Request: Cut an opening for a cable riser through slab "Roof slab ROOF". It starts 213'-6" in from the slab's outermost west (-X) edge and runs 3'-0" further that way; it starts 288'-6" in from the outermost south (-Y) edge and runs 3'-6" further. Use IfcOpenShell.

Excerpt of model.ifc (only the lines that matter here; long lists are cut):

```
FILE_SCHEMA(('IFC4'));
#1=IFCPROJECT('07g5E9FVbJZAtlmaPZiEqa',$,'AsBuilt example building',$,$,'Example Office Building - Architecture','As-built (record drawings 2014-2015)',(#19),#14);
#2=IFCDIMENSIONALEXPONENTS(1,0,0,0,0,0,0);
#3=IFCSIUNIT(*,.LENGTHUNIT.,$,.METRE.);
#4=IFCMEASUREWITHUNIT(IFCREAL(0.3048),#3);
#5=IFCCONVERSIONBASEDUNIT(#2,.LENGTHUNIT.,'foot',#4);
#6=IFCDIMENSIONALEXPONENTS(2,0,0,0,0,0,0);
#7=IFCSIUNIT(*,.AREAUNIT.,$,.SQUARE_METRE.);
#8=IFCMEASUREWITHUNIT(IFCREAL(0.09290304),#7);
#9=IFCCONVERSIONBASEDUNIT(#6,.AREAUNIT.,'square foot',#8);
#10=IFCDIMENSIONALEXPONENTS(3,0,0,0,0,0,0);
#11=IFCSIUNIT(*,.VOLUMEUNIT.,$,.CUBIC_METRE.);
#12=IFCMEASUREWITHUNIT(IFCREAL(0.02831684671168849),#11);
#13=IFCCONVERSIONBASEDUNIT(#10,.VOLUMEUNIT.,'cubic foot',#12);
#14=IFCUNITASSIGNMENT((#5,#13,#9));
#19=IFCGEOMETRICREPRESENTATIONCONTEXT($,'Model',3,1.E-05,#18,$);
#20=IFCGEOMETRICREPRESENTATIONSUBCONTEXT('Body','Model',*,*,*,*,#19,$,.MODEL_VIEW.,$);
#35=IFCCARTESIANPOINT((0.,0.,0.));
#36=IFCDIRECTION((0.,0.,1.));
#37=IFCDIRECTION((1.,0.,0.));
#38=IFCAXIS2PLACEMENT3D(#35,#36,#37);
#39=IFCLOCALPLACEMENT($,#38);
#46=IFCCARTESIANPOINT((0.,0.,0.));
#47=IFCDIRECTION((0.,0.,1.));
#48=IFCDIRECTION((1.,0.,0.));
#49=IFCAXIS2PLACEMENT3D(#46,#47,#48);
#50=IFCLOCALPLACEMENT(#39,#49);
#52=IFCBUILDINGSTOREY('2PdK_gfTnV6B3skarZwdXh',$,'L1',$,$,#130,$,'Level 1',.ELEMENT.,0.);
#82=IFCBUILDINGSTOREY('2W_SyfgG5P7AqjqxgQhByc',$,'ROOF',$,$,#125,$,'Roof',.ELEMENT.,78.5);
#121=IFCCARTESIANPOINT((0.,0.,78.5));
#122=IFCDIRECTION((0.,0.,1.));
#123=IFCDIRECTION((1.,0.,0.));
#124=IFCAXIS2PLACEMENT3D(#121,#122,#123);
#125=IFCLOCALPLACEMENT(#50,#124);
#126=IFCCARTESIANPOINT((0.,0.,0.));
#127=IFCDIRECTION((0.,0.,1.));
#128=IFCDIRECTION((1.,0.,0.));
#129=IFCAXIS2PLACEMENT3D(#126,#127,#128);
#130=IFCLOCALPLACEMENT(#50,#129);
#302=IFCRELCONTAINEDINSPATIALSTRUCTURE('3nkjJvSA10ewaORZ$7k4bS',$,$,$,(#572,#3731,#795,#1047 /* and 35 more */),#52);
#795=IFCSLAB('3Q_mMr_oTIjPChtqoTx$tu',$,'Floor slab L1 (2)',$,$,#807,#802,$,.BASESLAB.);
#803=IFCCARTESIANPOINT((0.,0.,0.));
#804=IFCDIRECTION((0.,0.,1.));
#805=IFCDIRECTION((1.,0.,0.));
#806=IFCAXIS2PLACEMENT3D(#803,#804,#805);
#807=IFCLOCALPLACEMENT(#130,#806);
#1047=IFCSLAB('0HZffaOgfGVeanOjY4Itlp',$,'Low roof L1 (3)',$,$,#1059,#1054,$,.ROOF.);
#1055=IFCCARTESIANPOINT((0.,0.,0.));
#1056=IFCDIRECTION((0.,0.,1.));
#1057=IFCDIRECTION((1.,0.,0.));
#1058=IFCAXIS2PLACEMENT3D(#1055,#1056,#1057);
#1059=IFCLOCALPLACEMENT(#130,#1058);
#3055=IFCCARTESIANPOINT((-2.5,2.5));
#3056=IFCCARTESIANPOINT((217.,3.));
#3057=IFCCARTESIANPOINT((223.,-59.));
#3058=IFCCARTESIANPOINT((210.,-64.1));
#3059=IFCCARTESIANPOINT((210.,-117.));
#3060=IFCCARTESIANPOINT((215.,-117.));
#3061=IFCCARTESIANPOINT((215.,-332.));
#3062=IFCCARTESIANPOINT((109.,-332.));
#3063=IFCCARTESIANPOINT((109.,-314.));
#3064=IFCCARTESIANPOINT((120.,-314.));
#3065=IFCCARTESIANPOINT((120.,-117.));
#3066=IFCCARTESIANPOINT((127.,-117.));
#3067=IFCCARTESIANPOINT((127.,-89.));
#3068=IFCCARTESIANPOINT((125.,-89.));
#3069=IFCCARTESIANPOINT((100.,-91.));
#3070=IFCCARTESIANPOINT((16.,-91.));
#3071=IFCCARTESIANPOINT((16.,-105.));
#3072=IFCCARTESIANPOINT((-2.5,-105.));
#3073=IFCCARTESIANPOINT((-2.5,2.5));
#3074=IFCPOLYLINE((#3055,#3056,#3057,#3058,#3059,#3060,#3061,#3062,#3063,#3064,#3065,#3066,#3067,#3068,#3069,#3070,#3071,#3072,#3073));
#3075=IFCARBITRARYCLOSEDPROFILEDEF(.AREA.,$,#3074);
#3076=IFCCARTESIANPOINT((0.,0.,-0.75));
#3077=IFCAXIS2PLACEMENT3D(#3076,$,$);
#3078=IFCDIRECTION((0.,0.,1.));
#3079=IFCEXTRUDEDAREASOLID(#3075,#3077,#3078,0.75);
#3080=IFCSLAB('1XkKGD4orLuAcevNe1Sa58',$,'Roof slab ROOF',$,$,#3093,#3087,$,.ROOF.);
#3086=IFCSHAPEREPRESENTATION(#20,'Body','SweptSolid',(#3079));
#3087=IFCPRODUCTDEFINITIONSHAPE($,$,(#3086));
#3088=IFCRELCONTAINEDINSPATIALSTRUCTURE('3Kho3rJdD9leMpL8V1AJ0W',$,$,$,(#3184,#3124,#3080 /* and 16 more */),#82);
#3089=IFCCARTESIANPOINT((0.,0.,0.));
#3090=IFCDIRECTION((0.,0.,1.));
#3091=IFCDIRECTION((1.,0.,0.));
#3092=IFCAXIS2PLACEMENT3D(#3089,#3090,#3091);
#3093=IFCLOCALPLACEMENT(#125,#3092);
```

```python
import numpy as np
import ifcopenshell
import ifcopenshell.api.feature
import ifcopenshell.api.geometry
import ifcopenshell.api.root
import ifcopenshell.geom
import ifcopenshell.util.placement
import ifcopenshell.util.representation
import ifcopenshell.util.shape
import ifcopenshell.util.unit

model = ifcopenshell.open("model.ifc")
unit_scale = ifcopenshell.util.unit.calculate_unit_scale(model)
settings = ifcopenshell.geom.settings()


def volume(element):
    """Net volume in cubic metres, openings subtracted."""
    shape = ifcopenshell.geom.create_shape(settings, element)
    return ifcopenshell.util.shape.get_volume(shape.geometry)


slab = model.by_guid("1XkKGD4orLuAcevNe1Sa58")
before = volume(slab)

# Extent in the slab's own axes, in metres. The edges named are its -X and -Y sides.
slab_shape = ifcopenshell.geom.create_shape(settings, slab)
vertices = ifcopenshell.util.shape.get_vertices(slab_shape.geometry)
x_min, y_min, bottom = vertices.min(axis=0)
top = vertices[:, 2].max()

opening = ifcopenshell.api.root.create_entity(model, ifc_class="IfcOpeningElement", name="Cable riser opening", predefined_type="OPENING")
context = ifcopenshell.util.representation.get_context(model, "Model", "Body", "MODEL_VIEW")
width, depth = 0.9144, 1.0668
outline = [(0.0, 0.0), (width, 0.0), (width, depth), (0.0, depth), (0.0, 0.0)]
# Overshoot both faces by 50 mm so the cut is clean.
shape = ifcopenshell.api.geometry.add_slab_representation(
    model, context=context, depth=top - bottom + 0.1, polyline=outline
)
ifcopenshell.api.geometry.assign_representation(model, product=opening, representation=shape)

matrix = ifcopenshell.util.placement.get_local_placement(slab.ObjectPlacement)
matrix[:, 3] = matrix @ np.append(np.array([x_min + 65.0748, y_min + 87.9348, bottom - 0.05]) / unit_scale, 1.0)
ifcopenshell.api.geometry.edit_object_placement(model, product=opening, matrix=matrix, is_si=False)
ifcopenshell.api.feature.add_feature(model, feature=opening, element=slab)

after = volume(slab)

print(f"slab volume {before:.3f} -> {after:.3f} m3")

model.write("model_v2.ifc")
```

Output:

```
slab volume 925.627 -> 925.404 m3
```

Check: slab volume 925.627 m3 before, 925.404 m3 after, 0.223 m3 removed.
